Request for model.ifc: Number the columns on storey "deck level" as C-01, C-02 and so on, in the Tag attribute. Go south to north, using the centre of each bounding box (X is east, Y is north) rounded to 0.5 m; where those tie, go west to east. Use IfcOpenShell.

First a look at what the model holds.

```python
import ifcopenshell
import ifcopenshell.util.element
import ifcopenshell.util.placement

model = ifcopenshell.open("model.ifc")
print(model.schema)
storey = next(s for s in model.by_type("IfcBuildingStorey") if s.Name == "deck level")
columns = [e for e in ifcopenshell.util.element.get_decomposition(storey) if e.is_a("IfcColumn")]
for e in sorted(columns, key=lambda e: e.id()):
    origin = ifcopenshell.util.placement.get_local_placement(e.ObjectPlacement)[:3, 3]
    print(e.id(), e.Tag, e.Name, origin.round(2) + 0.0, sep=" | ")
```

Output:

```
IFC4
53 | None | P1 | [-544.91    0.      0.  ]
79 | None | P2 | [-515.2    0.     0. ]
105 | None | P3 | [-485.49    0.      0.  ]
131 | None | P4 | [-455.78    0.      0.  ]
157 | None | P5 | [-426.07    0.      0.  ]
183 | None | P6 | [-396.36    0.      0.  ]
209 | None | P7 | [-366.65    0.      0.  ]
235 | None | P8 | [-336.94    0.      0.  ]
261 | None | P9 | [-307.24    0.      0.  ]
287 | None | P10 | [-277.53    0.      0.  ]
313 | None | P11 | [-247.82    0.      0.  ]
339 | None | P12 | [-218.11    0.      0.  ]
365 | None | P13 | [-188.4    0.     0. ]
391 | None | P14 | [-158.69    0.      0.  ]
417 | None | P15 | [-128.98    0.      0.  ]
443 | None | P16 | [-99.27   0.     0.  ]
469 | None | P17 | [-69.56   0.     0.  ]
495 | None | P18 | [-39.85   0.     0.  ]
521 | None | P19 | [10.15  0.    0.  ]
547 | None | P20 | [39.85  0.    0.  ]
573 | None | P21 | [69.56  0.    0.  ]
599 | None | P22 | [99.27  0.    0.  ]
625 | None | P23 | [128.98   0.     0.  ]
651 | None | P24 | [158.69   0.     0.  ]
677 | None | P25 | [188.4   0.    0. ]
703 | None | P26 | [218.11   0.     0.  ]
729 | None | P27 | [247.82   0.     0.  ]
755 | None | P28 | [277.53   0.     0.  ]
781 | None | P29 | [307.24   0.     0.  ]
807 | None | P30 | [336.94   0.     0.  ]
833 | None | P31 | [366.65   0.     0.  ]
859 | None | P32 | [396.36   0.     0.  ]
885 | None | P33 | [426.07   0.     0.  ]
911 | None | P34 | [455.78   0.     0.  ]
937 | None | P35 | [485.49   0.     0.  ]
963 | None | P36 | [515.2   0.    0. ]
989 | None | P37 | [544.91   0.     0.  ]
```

```python
import ifcopenshell
import ifcopenshell.geom
import ifcopenshell.util.element
import ifcopenshell.util.shape

model = ifcopenshell.open("model.ifc")
settings = ifcopenshell.geom.settings()
settings.set("use-world-coords", True)


def centre(element):
    shape = ifcopenshell.geom.create_shape(settings, element)
    return ifcopenshell.util.shape.get_bbox_centroid(shape.geometry)


storey = next(s for s in model.by_type("IfcBuildingStorey") if s.Name == "deck level")
columns = [e for e in ifcopenshell.util.element.get_decomposition(storey) if e.is_a("IfcColumn")]

# Insertion points can sit at a corner or the storey origin, so sort by the geometry (in metres).
centres = {e: centre(e) for e in columns}
columns.sort(key=lambda e: (round(centres[e][1] / 0.5), centres[e][0]))

for i, e in enumerate(columns, start=1):
    number = f"C-{i:02d}"
    e.Tag = number
    print(e.id(), number)

model.write("model_updated.ifc")
```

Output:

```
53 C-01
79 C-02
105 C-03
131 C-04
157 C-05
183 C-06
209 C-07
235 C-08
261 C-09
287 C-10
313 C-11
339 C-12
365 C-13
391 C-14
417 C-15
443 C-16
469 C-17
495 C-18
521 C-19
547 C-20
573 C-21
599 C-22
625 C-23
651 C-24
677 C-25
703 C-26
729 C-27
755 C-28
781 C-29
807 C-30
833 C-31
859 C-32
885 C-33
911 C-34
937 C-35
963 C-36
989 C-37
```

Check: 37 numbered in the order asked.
